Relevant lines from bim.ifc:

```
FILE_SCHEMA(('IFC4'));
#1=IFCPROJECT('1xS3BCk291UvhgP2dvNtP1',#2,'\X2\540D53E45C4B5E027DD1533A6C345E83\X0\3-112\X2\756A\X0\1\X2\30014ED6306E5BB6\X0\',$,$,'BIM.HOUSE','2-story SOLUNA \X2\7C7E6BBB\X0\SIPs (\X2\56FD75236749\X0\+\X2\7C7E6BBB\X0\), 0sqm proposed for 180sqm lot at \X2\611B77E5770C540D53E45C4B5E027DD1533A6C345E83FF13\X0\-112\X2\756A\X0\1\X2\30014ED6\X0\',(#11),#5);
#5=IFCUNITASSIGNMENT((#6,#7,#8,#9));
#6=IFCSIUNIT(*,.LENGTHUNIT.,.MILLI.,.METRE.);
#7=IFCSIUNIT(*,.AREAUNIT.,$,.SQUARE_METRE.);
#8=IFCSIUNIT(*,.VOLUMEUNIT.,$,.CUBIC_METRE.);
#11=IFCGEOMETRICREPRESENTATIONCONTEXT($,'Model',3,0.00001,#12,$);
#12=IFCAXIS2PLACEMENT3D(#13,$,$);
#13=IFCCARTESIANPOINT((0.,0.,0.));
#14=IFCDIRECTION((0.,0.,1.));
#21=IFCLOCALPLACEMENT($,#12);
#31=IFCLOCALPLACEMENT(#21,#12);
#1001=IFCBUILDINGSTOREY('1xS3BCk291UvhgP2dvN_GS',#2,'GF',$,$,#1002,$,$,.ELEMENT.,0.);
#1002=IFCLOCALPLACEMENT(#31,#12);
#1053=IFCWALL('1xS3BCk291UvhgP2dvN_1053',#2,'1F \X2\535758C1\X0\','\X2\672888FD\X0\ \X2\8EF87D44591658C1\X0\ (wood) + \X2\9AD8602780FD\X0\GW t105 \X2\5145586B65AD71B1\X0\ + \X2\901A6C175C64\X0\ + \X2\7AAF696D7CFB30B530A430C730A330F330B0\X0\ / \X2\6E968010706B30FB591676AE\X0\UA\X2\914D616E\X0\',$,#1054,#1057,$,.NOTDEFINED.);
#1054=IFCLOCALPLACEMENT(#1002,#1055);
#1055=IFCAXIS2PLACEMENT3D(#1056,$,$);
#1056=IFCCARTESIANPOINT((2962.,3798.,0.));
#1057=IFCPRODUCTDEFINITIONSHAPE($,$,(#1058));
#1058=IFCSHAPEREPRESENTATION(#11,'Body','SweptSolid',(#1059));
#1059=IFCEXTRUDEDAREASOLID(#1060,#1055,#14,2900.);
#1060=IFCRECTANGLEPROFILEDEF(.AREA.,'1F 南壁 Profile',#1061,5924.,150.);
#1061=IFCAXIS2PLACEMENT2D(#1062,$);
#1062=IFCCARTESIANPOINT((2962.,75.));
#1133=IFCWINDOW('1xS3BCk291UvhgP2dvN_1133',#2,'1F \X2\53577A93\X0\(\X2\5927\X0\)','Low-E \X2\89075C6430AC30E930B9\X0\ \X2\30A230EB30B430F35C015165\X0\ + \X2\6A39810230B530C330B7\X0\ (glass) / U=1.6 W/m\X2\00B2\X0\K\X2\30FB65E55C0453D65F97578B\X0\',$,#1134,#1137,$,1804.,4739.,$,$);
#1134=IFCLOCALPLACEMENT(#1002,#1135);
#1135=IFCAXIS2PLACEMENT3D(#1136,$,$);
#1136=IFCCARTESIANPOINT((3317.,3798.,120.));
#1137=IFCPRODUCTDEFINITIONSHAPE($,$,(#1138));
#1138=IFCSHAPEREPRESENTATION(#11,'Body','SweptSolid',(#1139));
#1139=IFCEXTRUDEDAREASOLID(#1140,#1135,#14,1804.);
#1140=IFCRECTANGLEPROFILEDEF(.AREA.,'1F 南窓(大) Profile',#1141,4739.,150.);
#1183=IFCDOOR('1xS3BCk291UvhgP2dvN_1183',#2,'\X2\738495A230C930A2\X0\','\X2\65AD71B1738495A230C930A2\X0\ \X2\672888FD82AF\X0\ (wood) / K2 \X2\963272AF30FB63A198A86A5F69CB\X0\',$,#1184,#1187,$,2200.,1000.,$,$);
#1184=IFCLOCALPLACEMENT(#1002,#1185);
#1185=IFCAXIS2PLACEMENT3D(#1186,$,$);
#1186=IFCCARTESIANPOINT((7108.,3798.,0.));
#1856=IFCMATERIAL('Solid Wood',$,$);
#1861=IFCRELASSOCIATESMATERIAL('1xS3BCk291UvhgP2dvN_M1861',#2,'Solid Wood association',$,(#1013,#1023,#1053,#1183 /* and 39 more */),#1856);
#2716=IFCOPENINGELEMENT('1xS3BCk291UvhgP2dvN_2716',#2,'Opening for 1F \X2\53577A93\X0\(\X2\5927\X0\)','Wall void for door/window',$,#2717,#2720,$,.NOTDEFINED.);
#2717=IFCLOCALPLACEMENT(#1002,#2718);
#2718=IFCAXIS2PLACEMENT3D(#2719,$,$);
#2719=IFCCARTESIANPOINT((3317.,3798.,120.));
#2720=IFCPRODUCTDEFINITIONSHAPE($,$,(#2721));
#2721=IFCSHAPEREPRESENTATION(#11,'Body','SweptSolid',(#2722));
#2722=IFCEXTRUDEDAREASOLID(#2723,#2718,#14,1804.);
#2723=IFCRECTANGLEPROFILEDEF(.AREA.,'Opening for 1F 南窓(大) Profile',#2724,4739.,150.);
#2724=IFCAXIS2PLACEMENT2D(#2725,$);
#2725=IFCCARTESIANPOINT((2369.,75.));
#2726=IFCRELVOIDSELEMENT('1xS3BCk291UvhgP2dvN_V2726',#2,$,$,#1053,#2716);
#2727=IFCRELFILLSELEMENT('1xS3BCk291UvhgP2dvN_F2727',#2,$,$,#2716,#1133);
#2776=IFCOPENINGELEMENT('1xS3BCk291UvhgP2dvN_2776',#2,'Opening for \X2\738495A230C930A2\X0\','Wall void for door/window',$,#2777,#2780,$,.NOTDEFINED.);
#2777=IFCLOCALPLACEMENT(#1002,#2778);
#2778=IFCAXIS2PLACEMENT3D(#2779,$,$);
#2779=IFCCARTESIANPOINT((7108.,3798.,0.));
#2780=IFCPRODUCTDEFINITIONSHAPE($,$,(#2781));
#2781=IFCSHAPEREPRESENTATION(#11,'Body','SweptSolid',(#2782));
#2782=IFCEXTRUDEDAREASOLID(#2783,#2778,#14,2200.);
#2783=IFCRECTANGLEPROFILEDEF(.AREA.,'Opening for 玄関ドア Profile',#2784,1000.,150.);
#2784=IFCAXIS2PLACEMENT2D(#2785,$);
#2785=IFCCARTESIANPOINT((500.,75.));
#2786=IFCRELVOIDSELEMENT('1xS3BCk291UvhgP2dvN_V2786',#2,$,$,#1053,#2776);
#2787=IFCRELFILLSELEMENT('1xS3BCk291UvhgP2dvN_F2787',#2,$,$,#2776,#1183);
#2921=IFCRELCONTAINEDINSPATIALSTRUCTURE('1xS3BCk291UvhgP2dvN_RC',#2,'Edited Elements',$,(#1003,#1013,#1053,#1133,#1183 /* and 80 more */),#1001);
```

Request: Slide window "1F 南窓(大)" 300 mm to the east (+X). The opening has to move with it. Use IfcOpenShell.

```python
import ifcopenshell
import ifcopenshell.api.geometry
import ifcopenshell.util.placement
import ifcopenshell.util.unit

model = ifcopenshell.open("bim.ifc")
unit_scale = ifcopenshell.util.unit.calculate_unit_scale(model)

window = model.by_guid("1xS3BCk291UvhgP2dvN_1133")
opening = window.FillsVoids[0].RelatingOpeningElement
wall = opening.VoidsElements[0].RelatingBuildingElement

wall_matrix = ifcopenshell.util.placement.get_local_placement(wall.ObjectPlacement)
shift = wall_matrix[:3, 0] * 0.3 / unit_scale
before = ifcopenshell.util.placement.get_local_placement(window.ObjectPlacement)[:3, 3].copy()

# The window is not placed relative to its opening, so move both.
for product in (opening, window):
    matrix = ifcopenshell.util.placement.get_local_placement(product.ObjectPlacement)
    matrix[:3, 3] += shift
    ifcopenshell.api.geometry.edit_object_placement(model, product=product, matrix=matrix, is_si=False)

after = ifcopenshell.util.placement.get_local_placement(window.ObjectPlacement)[:3, 3]
print("window moved by", (after - before).round(3) + 0.0)

model.write("bim_updated.ifc")
```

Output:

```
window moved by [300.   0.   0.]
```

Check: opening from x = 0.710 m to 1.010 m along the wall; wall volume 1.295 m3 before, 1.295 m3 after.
